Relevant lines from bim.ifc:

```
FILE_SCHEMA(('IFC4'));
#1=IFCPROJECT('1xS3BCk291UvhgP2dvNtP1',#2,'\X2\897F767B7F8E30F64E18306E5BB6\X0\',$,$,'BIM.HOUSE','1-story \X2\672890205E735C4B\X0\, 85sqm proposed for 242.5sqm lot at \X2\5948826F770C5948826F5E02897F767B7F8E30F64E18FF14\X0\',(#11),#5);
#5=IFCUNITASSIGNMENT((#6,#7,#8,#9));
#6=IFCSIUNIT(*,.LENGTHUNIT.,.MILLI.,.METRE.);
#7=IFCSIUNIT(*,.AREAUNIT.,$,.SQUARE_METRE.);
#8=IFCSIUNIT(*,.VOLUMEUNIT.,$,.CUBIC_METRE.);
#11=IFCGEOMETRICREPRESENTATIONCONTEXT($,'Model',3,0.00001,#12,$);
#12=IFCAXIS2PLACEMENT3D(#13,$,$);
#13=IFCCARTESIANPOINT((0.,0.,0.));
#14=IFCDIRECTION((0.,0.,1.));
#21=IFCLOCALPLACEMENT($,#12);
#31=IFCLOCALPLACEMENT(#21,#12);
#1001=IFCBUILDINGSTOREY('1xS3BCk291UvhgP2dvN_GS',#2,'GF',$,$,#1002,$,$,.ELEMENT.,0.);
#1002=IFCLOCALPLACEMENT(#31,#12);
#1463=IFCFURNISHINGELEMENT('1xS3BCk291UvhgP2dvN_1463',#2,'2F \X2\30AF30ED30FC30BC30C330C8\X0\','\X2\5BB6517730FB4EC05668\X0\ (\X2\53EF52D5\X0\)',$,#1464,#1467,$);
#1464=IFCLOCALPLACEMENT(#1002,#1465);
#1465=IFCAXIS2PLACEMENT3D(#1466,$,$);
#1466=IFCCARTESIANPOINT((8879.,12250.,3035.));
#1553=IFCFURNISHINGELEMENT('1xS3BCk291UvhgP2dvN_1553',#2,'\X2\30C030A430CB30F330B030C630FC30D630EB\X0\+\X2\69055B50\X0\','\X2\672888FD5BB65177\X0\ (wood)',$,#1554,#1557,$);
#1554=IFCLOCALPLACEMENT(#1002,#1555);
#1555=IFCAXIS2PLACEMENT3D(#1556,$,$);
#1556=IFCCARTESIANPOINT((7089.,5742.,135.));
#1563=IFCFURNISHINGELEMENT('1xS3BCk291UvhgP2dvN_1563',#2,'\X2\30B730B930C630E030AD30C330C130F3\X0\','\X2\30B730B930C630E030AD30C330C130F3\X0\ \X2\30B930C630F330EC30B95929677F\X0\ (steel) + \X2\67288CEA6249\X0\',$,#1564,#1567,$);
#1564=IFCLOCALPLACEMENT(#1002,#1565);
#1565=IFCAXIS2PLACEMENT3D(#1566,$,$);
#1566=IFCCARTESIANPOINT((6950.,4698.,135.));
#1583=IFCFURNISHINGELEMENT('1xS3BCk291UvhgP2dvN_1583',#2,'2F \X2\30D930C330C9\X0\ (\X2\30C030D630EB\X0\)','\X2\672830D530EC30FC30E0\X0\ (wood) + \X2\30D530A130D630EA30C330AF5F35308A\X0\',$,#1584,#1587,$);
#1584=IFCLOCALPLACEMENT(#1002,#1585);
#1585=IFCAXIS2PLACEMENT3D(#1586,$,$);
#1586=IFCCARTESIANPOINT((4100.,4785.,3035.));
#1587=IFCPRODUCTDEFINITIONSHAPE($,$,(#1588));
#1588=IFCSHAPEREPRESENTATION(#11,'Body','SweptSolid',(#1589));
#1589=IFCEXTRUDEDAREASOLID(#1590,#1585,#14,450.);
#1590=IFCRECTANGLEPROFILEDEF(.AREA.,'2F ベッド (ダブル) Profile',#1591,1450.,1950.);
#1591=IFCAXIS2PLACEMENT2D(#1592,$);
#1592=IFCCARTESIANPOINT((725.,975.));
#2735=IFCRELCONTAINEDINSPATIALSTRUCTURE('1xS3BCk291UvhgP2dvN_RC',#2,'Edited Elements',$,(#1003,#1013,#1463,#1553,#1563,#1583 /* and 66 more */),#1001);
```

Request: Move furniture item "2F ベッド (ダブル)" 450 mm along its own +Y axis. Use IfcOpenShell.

```python
import ifcopenshell
import ifcopenshell.api.geometry
import ifcopenshell.util.placement

model = ifcopenshell.open("bim.ifc")

item = model.by_guid("1xS3BCk291UvhgP2dvN_1583")
matrix = ifcopenshell.util.placement.get_local_placement(item.ObjectPlacement)
matrix[:3, 3] += matrix[:3, 1] * 450.0
ifcopenshell.api.geometry.edit_object_placement(model, product=item, matrix=matrix, is_si=False)

print(ifcopenshell.util.placement.get_local_placement(item.ObjectPlacement).round(3) + 0.0)

model.write("bim_edited.ifc")
```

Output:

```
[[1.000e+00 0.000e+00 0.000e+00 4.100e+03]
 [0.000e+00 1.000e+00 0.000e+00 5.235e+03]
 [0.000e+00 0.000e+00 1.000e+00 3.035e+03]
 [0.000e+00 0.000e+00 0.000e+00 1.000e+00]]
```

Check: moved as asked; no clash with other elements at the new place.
